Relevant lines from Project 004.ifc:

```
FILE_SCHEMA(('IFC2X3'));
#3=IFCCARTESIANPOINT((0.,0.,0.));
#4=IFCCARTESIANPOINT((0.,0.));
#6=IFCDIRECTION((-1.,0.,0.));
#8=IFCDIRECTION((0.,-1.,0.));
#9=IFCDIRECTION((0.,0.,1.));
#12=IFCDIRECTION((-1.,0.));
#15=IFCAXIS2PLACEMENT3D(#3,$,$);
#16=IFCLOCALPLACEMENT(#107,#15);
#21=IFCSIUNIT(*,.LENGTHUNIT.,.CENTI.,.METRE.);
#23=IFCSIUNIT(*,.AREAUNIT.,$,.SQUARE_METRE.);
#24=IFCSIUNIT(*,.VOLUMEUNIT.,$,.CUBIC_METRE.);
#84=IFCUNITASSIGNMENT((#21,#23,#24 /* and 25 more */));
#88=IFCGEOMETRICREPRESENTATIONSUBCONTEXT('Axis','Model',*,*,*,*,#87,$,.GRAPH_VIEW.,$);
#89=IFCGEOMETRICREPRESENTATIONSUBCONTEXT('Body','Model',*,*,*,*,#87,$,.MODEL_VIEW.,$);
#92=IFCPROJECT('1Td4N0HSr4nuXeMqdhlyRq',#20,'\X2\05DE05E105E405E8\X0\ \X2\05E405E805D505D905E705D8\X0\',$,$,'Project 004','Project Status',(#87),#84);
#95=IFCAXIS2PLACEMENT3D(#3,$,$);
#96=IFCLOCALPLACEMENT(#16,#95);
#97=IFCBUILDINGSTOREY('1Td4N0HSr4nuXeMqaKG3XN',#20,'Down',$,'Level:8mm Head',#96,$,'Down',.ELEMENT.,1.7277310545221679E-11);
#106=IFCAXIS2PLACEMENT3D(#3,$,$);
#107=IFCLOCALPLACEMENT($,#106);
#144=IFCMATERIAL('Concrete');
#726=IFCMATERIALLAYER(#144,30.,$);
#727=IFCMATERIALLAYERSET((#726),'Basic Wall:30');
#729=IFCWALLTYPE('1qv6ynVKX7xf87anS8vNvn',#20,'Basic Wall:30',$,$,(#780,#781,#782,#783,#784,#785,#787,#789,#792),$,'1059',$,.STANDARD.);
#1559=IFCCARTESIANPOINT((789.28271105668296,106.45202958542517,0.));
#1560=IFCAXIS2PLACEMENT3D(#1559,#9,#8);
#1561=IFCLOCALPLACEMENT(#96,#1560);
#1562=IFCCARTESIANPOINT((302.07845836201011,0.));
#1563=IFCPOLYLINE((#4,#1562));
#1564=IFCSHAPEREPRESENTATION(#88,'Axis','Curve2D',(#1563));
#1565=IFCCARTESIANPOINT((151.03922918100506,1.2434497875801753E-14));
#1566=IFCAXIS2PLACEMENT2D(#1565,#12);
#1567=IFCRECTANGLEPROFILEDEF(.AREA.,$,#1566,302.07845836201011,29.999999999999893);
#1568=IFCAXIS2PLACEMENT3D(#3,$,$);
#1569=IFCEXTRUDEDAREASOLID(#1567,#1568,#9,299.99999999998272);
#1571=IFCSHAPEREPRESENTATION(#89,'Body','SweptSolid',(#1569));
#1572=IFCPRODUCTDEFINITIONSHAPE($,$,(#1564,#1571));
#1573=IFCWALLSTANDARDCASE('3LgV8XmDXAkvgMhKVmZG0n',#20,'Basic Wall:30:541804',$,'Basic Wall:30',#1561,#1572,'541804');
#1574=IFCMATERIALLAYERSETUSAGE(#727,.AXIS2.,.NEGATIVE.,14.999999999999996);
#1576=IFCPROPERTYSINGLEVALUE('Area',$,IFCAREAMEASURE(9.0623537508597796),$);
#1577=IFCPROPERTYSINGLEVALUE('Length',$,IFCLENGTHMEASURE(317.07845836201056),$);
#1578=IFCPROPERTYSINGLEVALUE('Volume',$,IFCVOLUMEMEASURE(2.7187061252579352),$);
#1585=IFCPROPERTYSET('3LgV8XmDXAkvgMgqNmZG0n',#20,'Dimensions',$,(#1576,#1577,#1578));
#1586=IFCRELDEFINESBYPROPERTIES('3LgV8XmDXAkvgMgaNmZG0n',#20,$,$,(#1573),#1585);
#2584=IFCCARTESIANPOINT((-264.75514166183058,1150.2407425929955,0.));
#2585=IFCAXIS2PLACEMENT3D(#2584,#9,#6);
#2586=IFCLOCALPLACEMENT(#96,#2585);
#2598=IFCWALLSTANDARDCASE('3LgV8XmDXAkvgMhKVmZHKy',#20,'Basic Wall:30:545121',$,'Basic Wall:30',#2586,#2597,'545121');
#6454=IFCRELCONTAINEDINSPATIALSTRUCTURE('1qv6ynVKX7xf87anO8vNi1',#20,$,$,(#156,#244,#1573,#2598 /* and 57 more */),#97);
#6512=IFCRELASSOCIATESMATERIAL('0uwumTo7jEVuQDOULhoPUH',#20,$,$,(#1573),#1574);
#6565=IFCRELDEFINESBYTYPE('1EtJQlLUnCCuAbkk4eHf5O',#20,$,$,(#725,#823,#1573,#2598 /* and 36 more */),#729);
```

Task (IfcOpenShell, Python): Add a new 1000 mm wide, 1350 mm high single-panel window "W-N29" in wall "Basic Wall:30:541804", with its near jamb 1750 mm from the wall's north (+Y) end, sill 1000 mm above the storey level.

```python
import numpy as np
import ifcopenshell
import ifcopenshell.api.feature
import ifcopenshell.api.geometry
import ifcopenshell.api.pset
import ifcopenshell.api.root
import ifcopenshell.api.spatial
import ifcopenshell.api.type
import ifcopenshell.geom
import ifcopenshell.util.element
import ifcopenshell.util.placement
import ifcopenshell.util.representation
import ifcopenshell.util.shape
import ifcopenshell.util.unit

model = ifcopenshell.open("Project 004.ifc")
unit_scale = ifcopenshell.util.unit.calculate_unit_scale(model)
area_scale = ifcopenshell.util.unit.calculate_unit_scale(model, "AREAUNIT")
volume_scale = ifcopenshell.util.unit.calculate_unit_scale(model, "VOLUMEUNIT")
settings = ifcopenshell.geom.settings()


def volume(element):
    """Net volume in cubic metres, openings subtracted."""
    shape = ifcopenshell.geom.create_shape(settings, element)
    return ifcopenshell.util.shape.get_volume(shape.geometry)


wall = model.by_guid("3LgV8XmDXAkvgMhKVmZG0n")
storey = ifcopenshell.util.element.get_container(wall, ifc_class="IfcBuildingStorey")
context = ifcopenshell.util.representation.get_context(model, "Model", "Body", "MODEL_VIEW")
before = volume(wall)

width, height, from_end, sill = 1, 1.35, 1.75, 1  # metres

# The wall runs along its own X axis, and the end named is its -X end.
wall_shape = ifcopenshell.geom.create_shape(settings, wall)
x, y, z = ifcopenshell.util.shape.get_vertices(wall_shape.geometry).T
start = x.min() + from_end
face, thickness = float(y.min()), float(y.max() - y.min())
wall_matrix = ifcopenshell.util.placement.get_local_placement(wall.ObjectPlacement)
level = ifcopenshell.util.placement.get_local_placement(storey.ObjectPlacement)[2, 3]


def in_wall(x, y):
    """Placement at x, y metres in the wall's axes, at sill height."""
    matrix = wall_matrix.copy()
    matrix[:, 3] = wall_matrix @ np.array([x / unit_scale, y / unit_scale, 0.0, 1.0])
    matrix[2, 3] = level + sill / unit_scale
    return matrix


# Opening: a box that overshoots both wall faces by 50 mm.
opening = ifcopenshell.api.root.create_entity(model, ifc_class="IfcOpeningElement")
box = ifcopenshell.api.geometry.add_wall_representation(
    model, context=context, length=width, height=height, thickness=thickness + 0.1
)
ifcopenshell.api.geometry.assign_representation(model, product=opening, representation=box)
ifcopenshell.api.geometry.edit_object_placement(model, product=opening, matrix=in_wall(start, face - 0.05), is_si=False)
ifcopenshell.api.feature.add_feature(model, feature=opening, element=wall)

window = ifcopenshell.api.root.create_entity(model, ifc_class="IfcWindow", name="W-N29")
window.OverallWidth, window.OverallHeight = width / unit_scale, height / unit_scale
body = ifcopenshell.api.geometry.add_window_representation(
    model,
    context=context,
    overall_width=window.OverallWidth,
    overall_height=window.OverallHeight,
    partition_type="SINGLE_PANEL",
)
ifcopenshell.api.geometry.assign_representation(model, product=window, representation=body)
ifcopenshell.api.spatial.assign_container(model, products=[window], relating_structure=storey)
fills = ifcopenshell.api.feature.add_filling(model, opening=opening, element=window)
fills.OwnerHistory = window.OwnerHistory  # required in IFC2X3

# IFC2X3 keeps the operation on the window style.
style = ifcopenshell.api.root.create_entity(model, ifc_class="IfcWindowStyle", name="W-N29")
style.OperationType, style.ConstructionType = "SINGLE_PANEL", "NOTDEFINED"
style.ParameterTakesPrecedence = style.Sizeable = False
ifcopenshell.api.type.assign_type(model, related_objects=[window], relating_type=style)

# Centre the window in the wall's thickness.
ifcopenshell.api.geometry.edit_object_placement(model, product=window, matrix=in_wall(start, face), is_si=False)
window_shape = ifcopenshell.geom.create_shape(settings, window)
depth = ifcopenshell.util.shape.get_vertices(window_shape.geometry)[:, 1]
offset = face + thickness / 2 - (depth.min() + depth.max()) / 2
ifcopenshell.api.geometry.edit_object_placement(model, product=window, matrix=in_wall(start, offset), is_si=False)

after = volume(wall)

# Update the wall's stored quantities.
pset = model.by_id(ifcopenshell.util.element.get_pset(wall, "Dimensions", should_inherit=False)["id"])
ifcopenshell.api.pset.edit_pset(model, pset=pset, properties={
    "Area": model.create_entity("IfcAreaMeasure", after / thickness / area_scale),
    "Volume": model.create_entity("IfcVolumeMeasure", after / volume_scale),
})

print(f"wall volume {before:.3f} -> {after:.3f} m3")

model.write("Project 004-out.ifc")
```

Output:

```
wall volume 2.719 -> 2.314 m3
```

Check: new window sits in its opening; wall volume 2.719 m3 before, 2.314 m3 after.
